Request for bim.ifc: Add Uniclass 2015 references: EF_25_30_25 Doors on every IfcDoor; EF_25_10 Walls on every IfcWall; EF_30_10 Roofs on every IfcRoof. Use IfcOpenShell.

First a look at what the model holds.

```python
import ifcopenshell

model = ifcopenshell.open("bim.ifc")
print(model.schema)
print("classifications:", [c.Name for c in model.by_type("IfcClassification")])
for ifc_class in ("IfcDoor", "IfcRoof", "IfcStair", "IfcWall", "IfcWindow"):
    print(ifc_class, len(model.by_type(ifc_class)))
```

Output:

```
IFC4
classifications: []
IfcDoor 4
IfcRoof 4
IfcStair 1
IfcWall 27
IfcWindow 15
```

```python
import ifcopenshell
import ifcopenshell.api.classification

model = ifcopenshell.open("bim.ifc")

system = ifcopenshell.api.classification.add_classification(model, classification="Uniclass 2015")

codes = {
    "IfcDoor": ("EF_25_30_25", "Doors"),
    "IfcWall": ("EF_25_10", "Walls"),
    "IfcRoof": ("EF_30_10", "Roofs"),
}
for ifc_class, (code, name) in codes.items():
    products = model.by_type(ifc_class)
    ifcopenshell.api.classification.add_reference(
        model, products=products, classification=system, identification=code, name=name
    )
    print(code, len(products))

model.write("bim_v2.ifc")
```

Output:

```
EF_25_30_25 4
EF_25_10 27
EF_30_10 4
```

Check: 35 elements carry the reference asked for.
